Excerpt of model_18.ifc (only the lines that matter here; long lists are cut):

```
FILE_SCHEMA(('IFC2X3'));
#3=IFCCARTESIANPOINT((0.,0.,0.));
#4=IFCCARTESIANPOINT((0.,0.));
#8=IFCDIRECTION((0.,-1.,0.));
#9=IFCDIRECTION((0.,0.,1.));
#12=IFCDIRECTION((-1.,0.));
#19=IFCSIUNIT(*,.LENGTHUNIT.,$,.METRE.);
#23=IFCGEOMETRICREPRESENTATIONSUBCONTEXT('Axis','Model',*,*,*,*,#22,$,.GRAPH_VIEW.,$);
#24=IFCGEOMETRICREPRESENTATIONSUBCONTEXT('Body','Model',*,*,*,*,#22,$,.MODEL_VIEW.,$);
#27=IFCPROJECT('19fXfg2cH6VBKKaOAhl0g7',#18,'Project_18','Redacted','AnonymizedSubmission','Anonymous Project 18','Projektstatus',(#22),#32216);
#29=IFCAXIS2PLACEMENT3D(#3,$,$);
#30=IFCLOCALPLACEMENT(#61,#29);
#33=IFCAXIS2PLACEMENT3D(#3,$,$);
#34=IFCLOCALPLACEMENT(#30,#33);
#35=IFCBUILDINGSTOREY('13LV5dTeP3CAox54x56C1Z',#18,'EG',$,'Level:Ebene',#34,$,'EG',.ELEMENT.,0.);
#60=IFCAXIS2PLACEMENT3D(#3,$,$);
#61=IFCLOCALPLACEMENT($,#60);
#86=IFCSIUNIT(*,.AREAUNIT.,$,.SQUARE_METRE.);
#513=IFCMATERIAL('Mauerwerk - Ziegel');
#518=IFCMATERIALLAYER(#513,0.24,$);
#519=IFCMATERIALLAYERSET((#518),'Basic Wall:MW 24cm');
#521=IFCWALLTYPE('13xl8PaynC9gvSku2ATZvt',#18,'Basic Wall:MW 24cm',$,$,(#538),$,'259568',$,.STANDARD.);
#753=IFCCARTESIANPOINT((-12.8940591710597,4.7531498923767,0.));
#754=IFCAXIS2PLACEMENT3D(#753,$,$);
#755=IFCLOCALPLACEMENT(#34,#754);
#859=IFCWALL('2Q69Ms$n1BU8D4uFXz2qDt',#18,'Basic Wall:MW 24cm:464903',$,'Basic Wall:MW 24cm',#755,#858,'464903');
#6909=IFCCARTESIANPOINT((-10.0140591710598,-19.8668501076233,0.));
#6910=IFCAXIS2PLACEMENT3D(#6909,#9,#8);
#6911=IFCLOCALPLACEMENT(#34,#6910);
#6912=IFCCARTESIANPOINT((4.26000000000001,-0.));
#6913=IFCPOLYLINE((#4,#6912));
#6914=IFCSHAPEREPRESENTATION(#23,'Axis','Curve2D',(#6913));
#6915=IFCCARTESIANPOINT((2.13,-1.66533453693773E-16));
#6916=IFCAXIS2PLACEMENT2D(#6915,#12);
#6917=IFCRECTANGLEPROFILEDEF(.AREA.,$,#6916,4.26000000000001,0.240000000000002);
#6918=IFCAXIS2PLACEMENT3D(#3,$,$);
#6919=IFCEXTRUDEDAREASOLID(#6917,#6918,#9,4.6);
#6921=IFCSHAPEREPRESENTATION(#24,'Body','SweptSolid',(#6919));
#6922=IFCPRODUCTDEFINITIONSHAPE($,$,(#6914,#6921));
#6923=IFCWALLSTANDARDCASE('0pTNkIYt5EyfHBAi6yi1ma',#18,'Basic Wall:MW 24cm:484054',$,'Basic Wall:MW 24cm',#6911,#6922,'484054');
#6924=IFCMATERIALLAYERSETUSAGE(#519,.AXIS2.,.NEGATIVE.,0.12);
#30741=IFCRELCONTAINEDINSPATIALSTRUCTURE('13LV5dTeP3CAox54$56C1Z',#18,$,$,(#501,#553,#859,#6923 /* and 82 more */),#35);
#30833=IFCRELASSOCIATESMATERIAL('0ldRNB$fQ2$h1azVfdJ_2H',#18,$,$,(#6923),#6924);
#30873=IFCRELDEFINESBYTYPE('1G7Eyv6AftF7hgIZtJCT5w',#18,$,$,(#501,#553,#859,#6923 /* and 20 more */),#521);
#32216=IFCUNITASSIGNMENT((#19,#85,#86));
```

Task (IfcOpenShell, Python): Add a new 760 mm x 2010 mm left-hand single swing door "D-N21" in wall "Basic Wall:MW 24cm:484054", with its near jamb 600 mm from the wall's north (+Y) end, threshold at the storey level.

```python
import numpy as np
import ifcopenshell
import ifcopenshell.api.feature
import ifcopenshell.api.geometry
import ifcopenshell.api.root
import ifcopenshell.api.spatial
import ifcopenshell.api.type
import ifcopenshell.geom
import ifcopenshell.util.element
import ifcopenshell.util.placement
import ifcopenshell.util.representation
import ifcopenshell.util.shape
import ifcopenshell.util.unit

model = ifcopenshell.open("model_18.ifc")
unit_scale = ifcopenshell.util.unit.calculate_unit_scale(model)
settings = ifcopenshell.geom.settings()


def volume(element):
    """Net volume in cubic metres, openings subtracted."""
    shape = ifcopenshell.geom.create_shape(settings, element)
    return ifcopenshell.util.shape.get_volume(shape.geometry)


wall = model.by_guid("0pTNkIYt5EyfHBAi6yi1ma")
storey = ifcopenshell.util.element.get_container(wall, ifc_class="IfcBuildingStorey")
context = ifcopenshell.util.representation.get_context(model, "Model", "Body", "MODEL_VIEW")
before = volume(wall)

width, height, from_end, sill = 0.76, 2.01, 0.6, 0.0  # metres

# The wall runs along its own X axis, and the end named is its -X end.
wall_shape = ifcopenshell.geom.create_shape(settings, wall)
x, y, z = ifcopenshell.util.shape.get_vertices(wall_shape.geometry).T
start = x.min() + from_end
face, thickness = float(y.min()), float(y.max() - y.min())
wall_matrix = ifcopenshell.util.placement.get_local_placement(wall.ObjectPlacement)
level = ifcopenshell.util.placement.get_local_placement(storey.ObjectPlacement)[2, 3]


def in_wall(x, y):
    """Placement at x, y metres in the wall's axes, at sill height."""
    matrix = wall_matrix.copy()
    matrix[:, 3] = wall_matrix @ np.array([x / unit_scale, y / unit_scale, 0.0, 1.0])
    matrix[2, 3] = level + sill / unit_scale
    return matrix


# Opening: a box that overshoots both wall faces by 50 mm.
opening = ifcopenshell.api.root.create_entity(model, ifc_class="IfcOpeningElement")
box = ifcopenshell.api.geometry.add_wall_representation(
    model, context=context, length=width, height=height, thickness=thickness + 0.1
)
ifcopenshell.api.geometry.assign_representation(model, product=opening, representation=box)
ifcopenshell.api.geometry.edit_object_placement(model, product=opening, matrix=in_wall(start, face - 0.05), is_si=False)
ifcopenshell.api.feature.add_feature(model, feature=opening, element=wall)

door = ifcopenshell.api.root.create_entity(model, ifc_class="IfcDoor", name="D-N21")
door.OverallWidth, door.OverallHeight = width / unit_scale, height / unit_scale
body = ifcopenshell.api.geometry.add_door_representation(
    model,
    context=context,
    overall_width=door.OverallWidth,
    overall_height=door.OverallHeight,
    operation_type="SINGLE_SWING_LEFT",
    lining_properties={"LiningDepth": thickness / unit_scale, "ThresholdDepth": thickness / unit_scale},
)
ifcopenshell.api.geometry.assign_representation(model, product=door, representation=body)
ifcopenshell.api.spatial.assign_container(model, products=[door], relating_structure=storey)
fills = ifcopenshell.api.feature.add_filling(model, opening=opening, element=door)
fills.OwnerHistory = door.OwnerHistory  # required in IFC2X3

# IFC2X3 keeps the operation on the door style.
style = ifcopenshell.api.root.create_entity(model, ifc_class="IfcDoorStyle", name="D-N21")
style.OperationType, style.ConstructionType = "SINGLE_SWING_LEFT", "NOTDEFINED"
style.ParameterTakesPrecedence = style.Sizeable = False
ifcopenshell.api.type.assign_type(model, related_objects=[door], relating_type=style)

# The lining spans the wall, so the door starts at the wall face.
ifcopenshell.api.geometry.edit_object_placement(model, product=door, matrix=in_wall(start, face), is_si=False)

after = volume(wall)

print(f"wall volume {before:.3f} -> {after:.3f} m3")

model.write("model_18_updated.ifc")
```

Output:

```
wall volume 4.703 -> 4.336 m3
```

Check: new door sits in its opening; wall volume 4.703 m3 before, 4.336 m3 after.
